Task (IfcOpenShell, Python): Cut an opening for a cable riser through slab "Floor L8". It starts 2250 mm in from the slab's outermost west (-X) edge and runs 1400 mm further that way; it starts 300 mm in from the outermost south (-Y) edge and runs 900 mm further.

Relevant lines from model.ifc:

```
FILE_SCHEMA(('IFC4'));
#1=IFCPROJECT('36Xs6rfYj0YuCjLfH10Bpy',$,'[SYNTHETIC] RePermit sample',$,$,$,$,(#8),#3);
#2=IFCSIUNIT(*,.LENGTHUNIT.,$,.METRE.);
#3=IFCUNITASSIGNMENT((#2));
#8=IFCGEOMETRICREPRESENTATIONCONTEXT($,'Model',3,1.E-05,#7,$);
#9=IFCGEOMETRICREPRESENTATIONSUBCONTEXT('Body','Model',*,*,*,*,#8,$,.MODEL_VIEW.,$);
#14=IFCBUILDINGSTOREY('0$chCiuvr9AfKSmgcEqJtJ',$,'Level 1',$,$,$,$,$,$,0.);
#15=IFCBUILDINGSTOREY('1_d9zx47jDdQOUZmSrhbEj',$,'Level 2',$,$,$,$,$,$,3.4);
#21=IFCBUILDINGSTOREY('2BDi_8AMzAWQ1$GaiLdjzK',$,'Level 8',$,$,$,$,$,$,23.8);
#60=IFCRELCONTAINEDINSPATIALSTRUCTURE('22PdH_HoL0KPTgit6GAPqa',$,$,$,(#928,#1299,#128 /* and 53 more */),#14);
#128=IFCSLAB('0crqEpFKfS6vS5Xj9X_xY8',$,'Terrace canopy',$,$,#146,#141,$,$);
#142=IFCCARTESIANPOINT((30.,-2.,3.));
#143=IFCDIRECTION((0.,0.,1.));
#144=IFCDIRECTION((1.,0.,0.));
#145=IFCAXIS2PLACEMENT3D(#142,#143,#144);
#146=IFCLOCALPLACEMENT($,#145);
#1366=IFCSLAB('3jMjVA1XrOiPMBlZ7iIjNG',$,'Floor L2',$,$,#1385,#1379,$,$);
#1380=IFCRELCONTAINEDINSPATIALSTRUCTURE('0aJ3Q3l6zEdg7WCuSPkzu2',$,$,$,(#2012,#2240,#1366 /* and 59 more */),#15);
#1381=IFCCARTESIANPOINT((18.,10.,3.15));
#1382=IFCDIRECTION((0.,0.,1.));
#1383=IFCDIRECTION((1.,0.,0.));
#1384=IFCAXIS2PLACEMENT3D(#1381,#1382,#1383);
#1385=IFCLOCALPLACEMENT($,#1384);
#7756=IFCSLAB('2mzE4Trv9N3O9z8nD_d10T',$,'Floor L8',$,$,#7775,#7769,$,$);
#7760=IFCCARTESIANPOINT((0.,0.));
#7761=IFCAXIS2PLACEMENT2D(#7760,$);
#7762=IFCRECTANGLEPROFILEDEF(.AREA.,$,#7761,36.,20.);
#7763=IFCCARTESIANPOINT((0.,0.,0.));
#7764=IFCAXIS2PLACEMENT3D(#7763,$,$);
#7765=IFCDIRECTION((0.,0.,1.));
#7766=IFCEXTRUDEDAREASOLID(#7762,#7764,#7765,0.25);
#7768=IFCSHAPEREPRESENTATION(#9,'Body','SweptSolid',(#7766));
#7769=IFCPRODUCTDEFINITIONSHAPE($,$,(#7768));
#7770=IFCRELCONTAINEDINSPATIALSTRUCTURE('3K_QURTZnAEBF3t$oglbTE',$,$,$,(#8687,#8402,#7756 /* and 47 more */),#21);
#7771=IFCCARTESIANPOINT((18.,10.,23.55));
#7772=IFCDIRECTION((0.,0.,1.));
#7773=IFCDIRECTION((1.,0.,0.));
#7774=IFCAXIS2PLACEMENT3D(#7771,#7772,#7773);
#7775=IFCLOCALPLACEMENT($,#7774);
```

```python
import numpy as np
import ifcopenshell
import ifcopenshell.api.feature
import ifcopenshell.api.geometry
import ifcopenshell.api.root
import ifcopenshell.geom
import ifcopenshell.util.placement
import ifcopenshell.util.representation
import ifcopenshell.util.shape
import ifcopenshell.util.unit

model = ifcopenshell.open("model.ifc")
unit_scale = ifcopenshell.util.unit.calculate_unit_scale(model)
settings = ifcopenshell.geom.settings()


def volume(element):
    """Net volume in cubic metres, openings subtracted."""
    shape = ifcopenshell.geom.create_shape(settings, element)
    return ifcopenshell.util.shape.get_volume(shape.geometry)


slab = model.by_guid("2mzE4Trv9N3O9z8nD_d10T")
before = volume(slab)

# Extent in the slab's own axes, in metres. The edges named are its -X and -Y sides.
slab_shape = ifcopenshell.geom.create_shape(settings, slab)
vertices = ifcopenshell.util.shape.get_vertices(slab_shape.geometry)
x_min, y_min, bottom = vertices.min(axis=0)
top = vertices[:, 2].max()

opening = ifcopenshell.api.root.create_entity(model, ifc_class="IfcOpeningElement", name="Cable riser opening", predefined_type="OPENING")
context = ifcopenshell.util.representation.get_context(model, "Model", "Body", "MODEL_VIEW")
width, depth = 1.4, 0.9
outline = [(0.0, 0.0), (width, 0.0), (width, depth), (0.0, depth), (0.0, 0.0)]
# Overshoot both faces by 50 mm so the cut is clean.
shape = ifcopenshell.api.geometry.add_slab_representation(
    model, context=context, depth=top - bottom + 0.1, polyline=outline
)
ifcopenshell.api.geometry.assign_representation(model, product=opening, representation=shape)

matrix = ifcopenshell.util.placement.get_local_placement(slab.ObjectPlacement)
matrix[:, 3] = matrix @ np.append(np.array([x_min + 2.25, y_min + 0.3, bottom - 0.05]) / unit_scale, 1.0)
ifcopenshell.api.geometry.edit_object_placement(model, product=opening, matrix=matrix, is_si=False)
ifcopenshell.api.feature.add_feature(model, feature=opening, element=slab)

after = volume(slab)

print(f"slab volume {before:.3f} -> {after:.3f} m3")

model.write("model_v2.ifc")
```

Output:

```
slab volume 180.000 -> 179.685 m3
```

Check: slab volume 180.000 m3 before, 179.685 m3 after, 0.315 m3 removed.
